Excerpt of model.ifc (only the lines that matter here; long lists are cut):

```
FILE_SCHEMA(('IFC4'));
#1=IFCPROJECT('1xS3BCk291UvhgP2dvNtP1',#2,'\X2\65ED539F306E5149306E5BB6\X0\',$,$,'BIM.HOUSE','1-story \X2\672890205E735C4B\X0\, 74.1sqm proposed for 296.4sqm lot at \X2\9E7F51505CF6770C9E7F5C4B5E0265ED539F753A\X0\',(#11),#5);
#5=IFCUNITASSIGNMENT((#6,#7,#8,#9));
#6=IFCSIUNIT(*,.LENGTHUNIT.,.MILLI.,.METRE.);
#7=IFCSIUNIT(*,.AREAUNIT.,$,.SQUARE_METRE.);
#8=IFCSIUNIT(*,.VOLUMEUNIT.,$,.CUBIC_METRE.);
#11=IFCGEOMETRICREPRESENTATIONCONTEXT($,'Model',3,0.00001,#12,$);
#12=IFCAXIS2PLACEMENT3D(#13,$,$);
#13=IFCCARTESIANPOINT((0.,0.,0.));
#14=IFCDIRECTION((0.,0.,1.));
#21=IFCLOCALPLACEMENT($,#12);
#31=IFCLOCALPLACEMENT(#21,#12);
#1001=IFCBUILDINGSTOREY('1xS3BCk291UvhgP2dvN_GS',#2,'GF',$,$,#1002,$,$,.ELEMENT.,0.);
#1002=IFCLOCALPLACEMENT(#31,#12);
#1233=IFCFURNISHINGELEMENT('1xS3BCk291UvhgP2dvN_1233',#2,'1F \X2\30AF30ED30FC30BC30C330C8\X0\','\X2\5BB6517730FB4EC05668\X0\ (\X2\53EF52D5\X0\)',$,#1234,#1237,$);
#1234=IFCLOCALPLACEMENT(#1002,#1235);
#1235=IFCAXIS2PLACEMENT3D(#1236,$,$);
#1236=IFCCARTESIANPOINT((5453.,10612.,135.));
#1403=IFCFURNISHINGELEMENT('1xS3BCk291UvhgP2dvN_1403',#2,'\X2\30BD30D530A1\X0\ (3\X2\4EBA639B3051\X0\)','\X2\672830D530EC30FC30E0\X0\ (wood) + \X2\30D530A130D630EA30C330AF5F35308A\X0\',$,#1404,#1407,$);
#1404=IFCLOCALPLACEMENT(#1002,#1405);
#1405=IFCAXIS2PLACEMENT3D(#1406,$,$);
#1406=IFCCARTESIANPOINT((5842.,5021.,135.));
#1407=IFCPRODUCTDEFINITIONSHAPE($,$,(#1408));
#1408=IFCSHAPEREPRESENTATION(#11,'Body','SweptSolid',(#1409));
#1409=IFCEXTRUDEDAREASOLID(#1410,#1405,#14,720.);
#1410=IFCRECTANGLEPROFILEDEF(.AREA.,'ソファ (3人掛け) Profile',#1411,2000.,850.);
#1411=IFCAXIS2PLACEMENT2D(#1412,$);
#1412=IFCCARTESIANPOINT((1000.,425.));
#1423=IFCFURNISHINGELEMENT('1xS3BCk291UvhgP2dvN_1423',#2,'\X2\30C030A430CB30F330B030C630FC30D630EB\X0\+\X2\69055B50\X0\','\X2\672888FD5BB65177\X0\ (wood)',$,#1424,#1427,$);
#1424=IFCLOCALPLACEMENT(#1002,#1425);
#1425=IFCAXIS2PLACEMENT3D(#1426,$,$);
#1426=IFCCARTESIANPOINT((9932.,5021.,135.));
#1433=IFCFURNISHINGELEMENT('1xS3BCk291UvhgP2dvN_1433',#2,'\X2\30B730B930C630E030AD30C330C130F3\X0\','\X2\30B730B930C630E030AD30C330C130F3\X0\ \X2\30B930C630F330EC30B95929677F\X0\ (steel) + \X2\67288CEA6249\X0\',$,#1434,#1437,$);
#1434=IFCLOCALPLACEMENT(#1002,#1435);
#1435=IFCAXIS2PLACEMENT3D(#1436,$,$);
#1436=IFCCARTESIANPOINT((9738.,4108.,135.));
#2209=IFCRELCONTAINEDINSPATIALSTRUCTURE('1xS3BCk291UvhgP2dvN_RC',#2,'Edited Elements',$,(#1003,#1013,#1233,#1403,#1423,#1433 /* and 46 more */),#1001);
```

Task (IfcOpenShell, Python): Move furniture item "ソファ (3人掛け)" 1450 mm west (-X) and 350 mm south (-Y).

```python
import ifcopenshell
import ifcopenshell.api.geometry
import ifcopenshell.util.placement

model = ifcopenshell.open("model.ifc")

item = model.by_id(1403)
matrix = ifcopenshell.util.placement.get_local_placement(item.ObjectPlacement)
matrix[0, 3] -= 1450.0
matrix[1, 3] -= 350.0
ifcopenshell.api.geometry.edit_object_placement(model, product=item, matrix=matrix, is_si=False)

print(ifcopenshell.util.placement.get_local_placement(item.ObjectPlacement).round(3) + 0.0)

model.write("model_updated.ifc")
```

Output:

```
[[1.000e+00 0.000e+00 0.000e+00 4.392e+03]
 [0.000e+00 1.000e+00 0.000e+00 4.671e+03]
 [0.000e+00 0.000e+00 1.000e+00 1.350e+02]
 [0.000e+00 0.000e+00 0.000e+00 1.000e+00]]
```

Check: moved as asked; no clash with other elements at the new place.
